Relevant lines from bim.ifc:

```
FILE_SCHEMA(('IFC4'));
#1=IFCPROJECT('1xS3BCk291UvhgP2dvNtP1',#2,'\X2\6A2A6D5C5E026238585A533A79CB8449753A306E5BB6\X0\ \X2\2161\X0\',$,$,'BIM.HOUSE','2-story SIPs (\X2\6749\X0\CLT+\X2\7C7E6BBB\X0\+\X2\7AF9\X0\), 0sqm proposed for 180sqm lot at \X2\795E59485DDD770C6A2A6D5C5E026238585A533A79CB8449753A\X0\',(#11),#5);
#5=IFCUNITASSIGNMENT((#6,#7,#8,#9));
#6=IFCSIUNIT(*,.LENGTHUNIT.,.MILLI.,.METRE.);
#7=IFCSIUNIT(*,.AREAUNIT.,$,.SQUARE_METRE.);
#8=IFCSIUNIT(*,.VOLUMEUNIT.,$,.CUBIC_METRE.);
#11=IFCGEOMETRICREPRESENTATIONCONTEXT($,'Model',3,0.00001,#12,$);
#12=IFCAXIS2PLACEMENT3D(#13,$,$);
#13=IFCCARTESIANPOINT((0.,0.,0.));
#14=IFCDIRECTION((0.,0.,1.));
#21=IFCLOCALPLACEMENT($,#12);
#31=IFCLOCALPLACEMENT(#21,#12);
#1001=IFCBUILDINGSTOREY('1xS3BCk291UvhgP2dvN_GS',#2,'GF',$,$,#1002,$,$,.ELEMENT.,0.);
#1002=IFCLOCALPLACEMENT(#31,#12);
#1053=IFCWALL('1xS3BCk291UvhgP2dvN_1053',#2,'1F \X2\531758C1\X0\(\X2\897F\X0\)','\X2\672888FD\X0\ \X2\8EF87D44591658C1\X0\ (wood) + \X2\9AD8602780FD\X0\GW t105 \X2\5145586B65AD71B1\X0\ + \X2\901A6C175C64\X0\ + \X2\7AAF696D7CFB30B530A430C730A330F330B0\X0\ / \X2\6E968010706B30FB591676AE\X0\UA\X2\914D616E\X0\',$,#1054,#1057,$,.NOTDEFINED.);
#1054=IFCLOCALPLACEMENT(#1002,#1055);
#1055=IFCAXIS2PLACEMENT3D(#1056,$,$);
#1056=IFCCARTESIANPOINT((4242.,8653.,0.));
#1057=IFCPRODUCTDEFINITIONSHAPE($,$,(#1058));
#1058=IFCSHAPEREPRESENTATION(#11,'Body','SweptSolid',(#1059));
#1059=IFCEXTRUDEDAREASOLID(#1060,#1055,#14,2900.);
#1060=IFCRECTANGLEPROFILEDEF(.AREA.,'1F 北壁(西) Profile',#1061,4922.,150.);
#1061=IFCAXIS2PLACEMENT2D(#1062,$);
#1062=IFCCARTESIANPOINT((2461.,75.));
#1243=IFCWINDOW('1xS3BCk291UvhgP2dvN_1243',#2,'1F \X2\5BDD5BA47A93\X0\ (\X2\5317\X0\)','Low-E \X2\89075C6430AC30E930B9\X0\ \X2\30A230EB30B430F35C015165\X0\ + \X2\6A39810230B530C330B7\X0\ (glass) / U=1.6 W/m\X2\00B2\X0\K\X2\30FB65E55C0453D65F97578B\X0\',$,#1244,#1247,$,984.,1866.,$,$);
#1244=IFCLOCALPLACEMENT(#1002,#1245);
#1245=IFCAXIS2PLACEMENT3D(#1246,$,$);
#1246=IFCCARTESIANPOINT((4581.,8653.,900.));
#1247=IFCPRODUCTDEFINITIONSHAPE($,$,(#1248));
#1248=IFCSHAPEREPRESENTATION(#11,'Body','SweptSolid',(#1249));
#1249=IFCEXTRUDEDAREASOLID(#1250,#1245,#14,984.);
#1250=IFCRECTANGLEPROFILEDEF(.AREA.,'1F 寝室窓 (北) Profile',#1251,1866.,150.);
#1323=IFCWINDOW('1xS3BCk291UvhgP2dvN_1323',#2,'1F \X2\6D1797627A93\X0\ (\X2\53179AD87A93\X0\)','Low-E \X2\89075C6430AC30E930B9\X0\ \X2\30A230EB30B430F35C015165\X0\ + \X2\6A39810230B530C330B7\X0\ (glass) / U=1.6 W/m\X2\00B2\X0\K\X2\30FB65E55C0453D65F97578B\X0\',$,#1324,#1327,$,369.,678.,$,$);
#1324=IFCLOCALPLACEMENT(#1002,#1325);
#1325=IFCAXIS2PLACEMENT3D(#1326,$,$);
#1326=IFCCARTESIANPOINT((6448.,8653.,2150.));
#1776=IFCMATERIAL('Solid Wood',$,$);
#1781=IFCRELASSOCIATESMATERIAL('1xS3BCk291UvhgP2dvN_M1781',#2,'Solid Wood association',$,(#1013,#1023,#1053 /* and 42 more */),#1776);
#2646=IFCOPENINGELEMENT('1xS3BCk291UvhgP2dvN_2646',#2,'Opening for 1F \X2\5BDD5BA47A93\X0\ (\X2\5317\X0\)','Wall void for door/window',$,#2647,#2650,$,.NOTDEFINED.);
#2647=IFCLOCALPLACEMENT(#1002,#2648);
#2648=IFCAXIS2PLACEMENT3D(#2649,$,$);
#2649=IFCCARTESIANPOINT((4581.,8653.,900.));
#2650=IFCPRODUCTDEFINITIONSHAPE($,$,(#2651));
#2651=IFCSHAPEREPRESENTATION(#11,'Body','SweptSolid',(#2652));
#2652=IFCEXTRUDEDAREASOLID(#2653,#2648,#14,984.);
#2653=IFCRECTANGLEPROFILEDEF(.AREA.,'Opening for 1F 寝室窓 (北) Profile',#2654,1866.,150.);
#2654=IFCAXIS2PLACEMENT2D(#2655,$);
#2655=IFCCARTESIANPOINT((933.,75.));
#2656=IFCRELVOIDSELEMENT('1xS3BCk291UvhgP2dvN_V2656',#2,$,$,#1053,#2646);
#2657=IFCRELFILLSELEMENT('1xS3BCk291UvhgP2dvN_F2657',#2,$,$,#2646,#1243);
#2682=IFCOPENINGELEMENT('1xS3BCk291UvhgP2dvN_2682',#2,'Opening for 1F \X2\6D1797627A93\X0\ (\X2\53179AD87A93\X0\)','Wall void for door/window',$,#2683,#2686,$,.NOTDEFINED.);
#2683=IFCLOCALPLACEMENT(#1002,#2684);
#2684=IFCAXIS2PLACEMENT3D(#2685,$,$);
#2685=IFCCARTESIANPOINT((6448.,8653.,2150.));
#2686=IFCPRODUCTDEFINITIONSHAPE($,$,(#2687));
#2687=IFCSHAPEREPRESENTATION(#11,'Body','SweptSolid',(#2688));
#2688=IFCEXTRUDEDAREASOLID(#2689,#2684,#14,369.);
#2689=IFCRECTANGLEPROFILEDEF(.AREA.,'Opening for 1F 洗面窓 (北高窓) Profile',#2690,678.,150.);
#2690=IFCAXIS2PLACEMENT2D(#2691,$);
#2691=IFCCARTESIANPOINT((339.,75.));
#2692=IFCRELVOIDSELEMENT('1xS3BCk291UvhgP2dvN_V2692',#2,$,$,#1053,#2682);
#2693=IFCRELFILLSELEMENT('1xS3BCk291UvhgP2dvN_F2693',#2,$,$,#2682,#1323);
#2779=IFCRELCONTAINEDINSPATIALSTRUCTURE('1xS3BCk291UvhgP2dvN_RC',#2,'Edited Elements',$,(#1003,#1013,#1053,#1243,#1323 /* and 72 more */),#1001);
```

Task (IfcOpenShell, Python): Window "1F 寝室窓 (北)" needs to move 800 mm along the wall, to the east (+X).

```python
import ifcopenshell
import ifcopenshell.api.geometry
import ifcopenshell.util.placement

model = ifcopenshell.open("bim.ifc")

window = model.by_guid("1xS3BCk291UvhgP2dvN_1243")
opening = window.FillsVoids[0].RelatingOpeningElement
wall = opening.VoidsElements[0].RelatingBuildingElement

wall_matrix = ifcopenshell.util.placement.get_local_placement(wall.ObjectPlacement)
shift = wall_matrix[:3, 0] * 800.0
before = ifcopenshell.util.placement.get_local_placement(window.ObjectPlacement)[:3, 3].copy()

# The window is not placed relative to its opening, so move both.
for product in (opening, window):
    matrix = ifcopenshell.util.placement.get_local_placement(product.ObjectPlacement)
    matrix[:3, 3] += shift
    ifcopenshell.api.geometry.edit_object_placement(model, product=product, matrix=matrix, is_si=False)

after = ifcopenshell.util.placement.get_local_placement(window.ObjectPlacement)[:3, 3]
print("window moved by", (after - before).round(3) + 0.0)

model.write("bim_updated.ifc")
```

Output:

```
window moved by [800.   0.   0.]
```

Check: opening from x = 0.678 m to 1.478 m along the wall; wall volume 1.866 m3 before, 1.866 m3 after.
